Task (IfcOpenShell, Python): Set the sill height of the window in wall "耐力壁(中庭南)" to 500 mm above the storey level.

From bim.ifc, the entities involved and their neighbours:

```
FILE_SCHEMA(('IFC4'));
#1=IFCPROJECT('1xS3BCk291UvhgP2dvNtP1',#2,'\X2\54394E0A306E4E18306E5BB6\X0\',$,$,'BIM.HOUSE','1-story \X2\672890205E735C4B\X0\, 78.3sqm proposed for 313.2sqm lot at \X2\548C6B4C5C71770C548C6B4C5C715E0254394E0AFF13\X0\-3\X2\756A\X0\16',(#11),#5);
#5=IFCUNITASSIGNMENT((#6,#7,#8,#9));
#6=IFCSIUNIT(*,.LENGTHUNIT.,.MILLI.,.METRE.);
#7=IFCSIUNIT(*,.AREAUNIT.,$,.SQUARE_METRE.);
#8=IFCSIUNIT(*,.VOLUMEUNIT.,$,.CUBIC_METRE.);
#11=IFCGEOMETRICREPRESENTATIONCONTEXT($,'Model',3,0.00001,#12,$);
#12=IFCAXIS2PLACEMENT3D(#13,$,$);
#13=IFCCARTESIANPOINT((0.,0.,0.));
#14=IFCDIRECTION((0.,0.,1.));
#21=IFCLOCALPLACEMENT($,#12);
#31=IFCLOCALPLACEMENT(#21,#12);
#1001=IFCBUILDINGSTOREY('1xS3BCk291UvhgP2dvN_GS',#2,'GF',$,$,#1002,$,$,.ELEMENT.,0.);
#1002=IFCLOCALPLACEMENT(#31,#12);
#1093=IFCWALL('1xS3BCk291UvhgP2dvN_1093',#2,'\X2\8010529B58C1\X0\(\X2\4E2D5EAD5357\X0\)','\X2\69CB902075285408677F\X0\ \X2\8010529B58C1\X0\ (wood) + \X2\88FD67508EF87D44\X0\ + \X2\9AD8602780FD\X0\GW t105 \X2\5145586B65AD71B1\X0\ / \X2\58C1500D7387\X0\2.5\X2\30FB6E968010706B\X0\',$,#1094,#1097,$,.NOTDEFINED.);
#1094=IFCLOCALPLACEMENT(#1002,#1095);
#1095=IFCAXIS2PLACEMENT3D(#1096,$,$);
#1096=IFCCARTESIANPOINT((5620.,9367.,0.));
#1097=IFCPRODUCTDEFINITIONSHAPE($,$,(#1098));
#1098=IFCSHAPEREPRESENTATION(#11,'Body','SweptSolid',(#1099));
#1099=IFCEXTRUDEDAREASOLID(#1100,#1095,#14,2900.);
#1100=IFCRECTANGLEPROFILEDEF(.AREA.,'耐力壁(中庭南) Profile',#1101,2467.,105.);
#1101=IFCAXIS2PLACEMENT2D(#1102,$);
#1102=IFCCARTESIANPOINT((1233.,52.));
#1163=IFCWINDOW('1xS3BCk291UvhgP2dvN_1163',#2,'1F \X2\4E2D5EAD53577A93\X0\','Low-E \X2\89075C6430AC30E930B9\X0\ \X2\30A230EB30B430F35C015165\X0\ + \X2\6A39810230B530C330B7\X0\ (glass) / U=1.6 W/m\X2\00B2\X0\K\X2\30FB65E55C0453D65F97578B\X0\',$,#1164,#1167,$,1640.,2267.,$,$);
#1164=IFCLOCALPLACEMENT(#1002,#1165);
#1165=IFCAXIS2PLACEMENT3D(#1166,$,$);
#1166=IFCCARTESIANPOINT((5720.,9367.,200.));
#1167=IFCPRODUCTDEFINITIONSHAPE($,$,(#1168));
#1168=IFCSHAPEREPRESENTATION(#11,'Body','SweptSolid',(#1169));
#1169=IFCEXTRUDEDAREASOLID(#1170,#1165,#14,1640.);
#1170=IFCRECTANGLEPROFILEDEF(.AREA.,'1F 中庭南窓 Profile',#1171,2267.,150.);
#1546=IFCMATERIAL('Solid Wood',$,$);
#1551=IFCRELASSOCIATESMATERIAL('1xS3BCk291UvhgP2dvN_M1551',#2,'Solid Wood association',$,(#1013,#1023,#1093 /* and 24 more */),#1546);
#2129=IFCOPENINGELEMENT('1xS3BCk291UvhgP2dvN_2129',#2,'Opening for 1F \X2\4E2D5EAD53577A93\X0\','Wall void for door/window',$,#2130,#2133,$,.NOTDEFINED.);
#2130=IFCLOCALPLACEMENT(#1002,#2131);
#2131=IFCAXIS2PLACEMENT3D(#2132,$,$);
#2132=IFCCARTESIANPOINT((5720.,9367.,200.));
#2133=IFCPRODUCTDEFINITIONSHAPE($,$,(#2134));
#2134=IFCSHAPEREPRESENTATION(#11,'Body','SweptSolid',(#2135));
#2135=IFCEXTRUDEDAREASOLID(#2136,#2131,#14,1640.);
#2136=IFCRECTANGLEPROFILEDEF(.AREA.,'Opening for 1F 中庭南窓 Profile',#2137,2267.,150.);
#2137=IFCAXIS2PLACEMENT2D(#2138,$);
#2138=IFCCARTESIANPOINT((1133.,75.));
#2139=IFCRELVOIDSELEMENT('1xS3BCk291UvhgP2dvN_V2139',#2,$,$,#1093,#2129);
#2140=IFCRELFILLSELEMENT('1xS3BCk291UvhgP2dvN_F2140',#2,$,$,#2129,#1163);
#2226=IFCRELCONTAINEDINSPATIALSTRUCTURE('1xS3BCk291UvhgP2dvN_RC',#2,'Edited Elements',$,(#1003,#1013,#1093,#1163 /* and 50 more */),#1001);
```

```python
import numpy as np
import ifcopenshell
import ifcopenshell.api.geometry
import ifcopenshell.geom
import ifcopenshell.util.element
import ifcopenshell.util.placement
import ifcopenshell.util.shape
import ifcopenshell.util.unit

model = ifcopenshell.open("bim.ifc")
unit_scale = ifcopenshell.util.unit.calculate_unit_scale(model)

window = model.by_guid("1xS3BCk291UvhgP2dvN_1163")
opening = window.FillsVoids[0].RelatingOpeningElement
storey = ifcopenshell.util.element.get_container(window, ifc_class="IfcBuildingStorey")
level = ifcopenshell.util.placement.get_local_placement(storey.ObjectPlacement)[2, 3]

# The opening's origin need not be at the sill, so measure its lowest point.
shape = ifcopenshell.geom.create_shape(ifcopenshell.geom.settings(), opening)
bottom = ifcopenshell.util.shape.get_shape_bottom_elevation(shape, shape.geometry) / unit_scale
dz = level + 500.0 - bottom

shift = np.array([0.0, 0.0, dz])
# The window is not placed relative to its opening, so move both.
for product in (opening, window):
    matrix = ifcopenshell.util.placement.get_local_placement(product.ObjectPlacement)
    matrix[:3, 3] += shift
    ifcopenshell.api.geometry.edit_object_placement(model, product=product, matrix=matrix, is_si=False)

print(f"moved by {dz * unit_scale:+.3f} m")

model.write("bim_v2.ifc")
```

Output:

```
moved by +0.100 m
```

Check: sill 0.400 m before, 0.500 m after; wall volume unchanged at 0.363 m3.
